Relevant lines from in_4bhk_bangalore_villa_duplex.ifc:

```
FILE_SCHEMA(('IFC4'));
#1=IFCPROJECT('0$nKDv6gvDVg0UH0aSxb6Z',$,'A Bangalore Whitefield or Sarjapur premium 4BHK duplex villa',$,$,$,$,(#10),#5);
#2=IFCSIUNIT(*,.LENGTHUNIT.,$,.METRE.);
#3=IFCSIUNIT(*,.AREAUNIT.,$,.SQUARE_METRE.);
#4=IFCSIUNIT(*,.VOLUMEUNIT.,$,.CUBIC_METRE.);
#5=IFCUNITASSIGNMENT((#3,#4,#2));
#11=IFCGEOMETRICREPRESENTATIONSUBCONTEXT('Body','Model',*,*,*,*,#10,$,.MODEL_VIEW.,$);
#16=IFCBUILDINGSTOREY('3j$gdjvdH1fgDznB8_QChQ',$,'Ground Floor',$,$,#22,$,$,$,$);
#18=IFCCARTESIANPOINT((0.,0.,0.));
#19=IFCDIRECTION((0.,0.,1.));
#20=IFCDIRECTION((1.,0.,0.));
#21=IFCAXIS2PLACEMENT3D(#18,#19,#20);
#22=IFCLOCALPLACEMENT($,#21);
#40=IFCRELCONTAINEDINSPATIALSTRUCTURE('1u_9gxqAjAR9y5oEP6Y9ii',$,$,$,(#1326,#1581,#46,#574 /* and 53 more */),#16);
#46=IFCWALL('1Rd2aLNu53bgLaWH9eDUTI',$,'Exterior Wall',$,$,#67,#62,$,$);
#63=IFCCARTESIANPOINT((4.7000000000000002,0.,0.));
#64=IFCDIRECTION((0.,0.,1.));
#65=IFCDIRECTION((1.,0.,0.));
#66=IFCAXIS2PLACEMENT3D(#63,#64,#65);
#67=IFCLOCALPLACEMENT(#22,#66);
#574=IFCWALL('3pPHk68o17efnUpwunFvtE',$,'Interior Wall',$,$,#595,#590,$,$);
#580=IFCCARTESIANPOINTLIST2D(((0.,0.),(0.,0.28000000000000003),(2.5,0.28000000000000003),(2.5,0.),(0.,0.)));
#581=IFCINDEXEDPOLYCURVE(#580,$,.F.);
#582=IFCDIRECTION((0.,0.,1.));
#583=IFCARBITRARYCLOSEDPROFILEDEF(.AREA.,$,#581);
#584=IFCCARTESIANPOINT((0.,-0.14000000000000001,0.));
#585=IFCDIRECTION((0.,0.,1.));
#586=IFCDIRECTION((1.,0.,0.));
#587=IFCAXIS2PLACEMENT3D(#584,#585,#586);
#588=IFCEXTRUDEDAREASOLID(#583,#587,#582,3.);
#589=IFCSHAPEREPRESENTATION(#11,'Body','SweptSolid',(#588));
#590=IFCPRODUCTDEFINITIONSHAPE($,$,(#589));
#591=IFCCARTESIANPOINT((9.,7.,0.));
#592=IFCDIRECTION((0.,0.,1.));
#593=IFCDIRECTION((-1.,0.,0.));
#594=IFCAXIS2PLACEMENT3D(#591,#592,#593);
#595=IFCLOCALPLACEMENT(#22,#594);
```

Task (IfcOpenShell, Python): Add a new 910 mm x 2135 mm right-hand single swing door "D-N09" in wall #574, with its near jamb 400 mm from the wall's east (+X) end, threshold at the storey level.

```python
import numpy as np
import ifcopenshell
import ifcopenshell.api.feature
import ifcopenshell.api.geometry
import ifcopenshell.api.root
import ifcopenshell.api.spatial
import ifcopenshell.geom
import ifcopenshell.util.element
import ifcopenshell.util.placement
import ifcopenshell.util.representation
import ifcopenshell.util.shape
import ifcopenshell.util.unit

model = ifcopenshell.open("in_4bhk_bangalore_villa_duplex.ifc")
unit_scale = ifcopenshell.util.unit.calculate_unit_scale(model)
settings = ifcopenshell.geom.settings()


def volume(element):
    """Net volume in cubic metres, openings subtracted."""
    shape = ifcopenshell.geom.create_shape(settings, element)
    return ifcopenshell.util.shape.get_volume(shape.geometry)


wall = model.by_guid("3pPHk68o17efnUpwunFvtE")
storey = ifcopenshell.util.element.get_container(wall, ifc_class="IfcBuildingStorey")
context = ifcopenshell.util.representation.get_context(model, "Model", "Body", "MODEL_VIEW")
before = volume(wall)

width, height, from_end, sill = 0.91, 2.135, 0.4, 0.0  # metres

# The wall runs along its own X axis, and the end named is its -X end.
wall_shape = ifcopenshell.geom.create_shape(settings, wall)
x, y, z = ifcopenshell.util.shape.get_vertices(wall_shape.geometry).T
start = x.min() + from_end
face, thickness = float(y.min()), float(y.max() - y.min())
wall_matrix = ifcopenshell.util.placement.get_local_placement(wall.ObjectPlacement)
level = ifcopenshell.util.placement.get_local_placement(storey.ObjectPlacement)[2, 3]


def in_wall(x, y):
    """Placement at x, y metres in the wall's axes, at sill height."""
    matrix = wall_matrix.copy()
    matrix[:, 3] = wall_matrix @ np.array([x / unit_scale, y / unit_scale, 0.0, 1.0])
    matrix[2, 3] = level + sill / unit_scale
    return matrix


# Opening: a box that overshoots both wall faces by 50 mm.
opening = ifcopenshell.api.root.create_entity(model, ifc_class="IfcOpeningElement", predefined_type="OPENING")
box = ifcopenshell.api.geometry.add_wall_representation(
    model, context=context, length=width, height=height, thickness=thickness + 0.1
)
ifcopenshell.api.geometry.assign_representation(model, product=opening, representation=box)
ifcopenshell.api.geometry.edit_object_placement(model, product=opening, matrix=in_wall(start, face - 0.05), is_si=False)
ifcopenshell.api.feature.add_feature(model, feature=opening, element=wall)

door = ifcopenshell.api.root.create_entity(model, ifc_class="IfcDoor", name="D-N09", predefined_type="DOOR")
door.OverallWidth, door.OverallHeight = width / unit_scale, height / unit_scale
door.OperationType = "SINGLE_SWING_RIGHT"
body = ifcopenshell.api.geometry.add_door_representation(
    model,
    context=context,
    overall_width=door.OverallWidth,
    overall_height=door.OverallHeight,
    operation_type="SINGLE_SWING_RIGHT",
    lining_properties={"LiningDepth": thickness / unit_scale, "ThresholdDepth": thickness / unit_scale},
)
ifcopenshell.api.geometry.assign_representation(model, product=door, representation=body)
ifcopenshell.api.spatial.assign_container(model, products=[door], relating_structure=storey)
ifcopenshell.api.feature.add_filling(model, opening=opening, element=door)

# The lining spans the wall, so the door starts at the wall face.
ifcopenshell.api.geometry.edit_object_placement(model, product=door, matrix=in_wall(start, face), is_si=False)

after = volume(wall)

print(f"wall volume {before:.3f} -> {after:.3f} m3")

model.write("in_4bhk_bangalore_villa_duplex_v2.ifc")
```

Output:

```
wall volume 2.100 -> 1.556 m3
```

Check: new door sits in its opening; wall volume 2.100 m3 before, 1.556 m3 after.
